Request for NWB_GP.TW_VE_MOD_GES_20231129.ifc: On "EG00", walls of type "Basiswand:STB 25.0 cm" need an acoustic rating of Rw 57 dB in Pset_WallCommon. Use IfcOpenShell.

First a look at what the model holds.

```python
import ifcopenshell
import ifcopenshell.util.element

model = ifcopenshell.open("NWB_GP.TW_VE_MOD_GES_20231129.ifc")
print(model.schema)
storey = next(s for s in model.by_type("IfcBuildingStorey") if s.Name == "EG00")
walls = [e for e in ifcopenshell.util.element.get_decomposition(storey) if e.is_a("IfcWall")]
seen = {}
for e in walls:
    element_type = ifcopenshell.util.element.get_type(e)
    key = (element_type.Name if element_type != e and element_type else None, ifcopenshell.util.element.get_pset(e, "Pset_WallCommon", "AcousticRating"))
    seen[key] = seen.get(key, 0) + 1
for (name, value), count in sorted(seen.items(), key=str):
    print(count, "x", name, "|", value)
```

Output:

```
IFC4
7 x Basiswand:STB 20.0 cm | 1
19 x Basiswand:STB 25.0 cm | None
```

```python
import ifcopenshell
import ifcopenshell.api.pset
import ifcopenshell.util.element

model = ifcopenshell.open("NWB_GP.TW_VE_MOD_GES_20231129.ifc")

storey = next(s for s in model.by_type("IfcBuildingStorey") if s.Name == "EG00")
walls = [e for e in ifcopenshell.util.element.get_decomposition(storey) if e.is_a("IfcWall")]

count = 0
for e in walls:
    element_type = ifcopenshell.util.element.get_type(e)
    if element_type in (None, e) or element_type.Name != "Basiswand:STB 25.0 cm":
        continue
    # add_pset returns the element's existing set when there is one.
    pset = ifcopenshell.api.pset.add_pset(model, product=e, name="Pset_WallCommon")
    ifcopenshell.api.pset.edit_pset(model, pset=pset, properties={"AcousticRating": "Rw 57 dB"})
    count += 1

print(count, "walls updated")

model.write("NWB_GP.TW_VE_MOD_GES_20231129_edited.ifc")
```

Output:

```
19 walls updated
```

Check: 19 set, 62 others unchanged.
